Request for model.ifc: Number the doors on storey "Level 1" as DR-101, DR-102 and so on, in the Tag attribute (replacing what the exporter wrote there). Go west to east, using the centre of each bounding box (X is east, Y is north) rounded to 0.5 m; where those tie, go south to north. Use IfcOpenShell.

First a look at what the model holds.

```python
import ifcopenshell
import ifcopenshell.util.element
import ifcopenshell.util.placement

model = ifcopenshell.open("model.ifc")
print(model.schema)
storey = next(s for s in model.by_type("IfcBuildingStorey") if s.Name == "Level 1")
doors = [e for e in ifcopenshell.util.element.get_decomposition(storey) if e.is_a("IfcDoor")]
for e in sorted(doors, key=lambda e: e.id()):
    origin = ifcopenshell.util.placement.get_local_placement(e.ObjectPlacement)[:3, 3]
    print(e.id(), e.Tag, e.Name, origin.round(2) + 0.0, sep=" | ")
```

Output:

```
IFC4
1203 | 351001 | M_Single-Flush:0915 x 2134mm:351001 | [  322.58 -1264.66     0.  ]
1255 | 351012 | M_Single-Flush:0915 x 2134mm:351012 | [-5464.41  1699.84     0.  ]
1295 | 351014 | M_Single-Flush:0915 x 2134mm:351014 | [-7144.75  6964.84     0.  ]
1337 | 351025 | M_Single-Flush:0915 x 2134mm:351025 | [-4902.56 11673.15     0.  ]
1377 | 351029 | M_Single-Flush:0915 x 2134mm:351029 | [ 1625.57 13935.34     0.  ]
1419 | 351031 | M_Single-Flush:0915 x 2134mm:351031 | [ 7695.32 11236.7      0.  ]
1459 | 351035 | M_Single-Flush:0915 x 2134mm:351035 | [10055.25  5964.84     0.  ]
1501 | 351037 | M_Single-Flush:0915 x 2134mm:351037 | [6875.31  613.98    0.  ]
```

```python
import ifcopenshell
import ifcopenshell.geom
import ifcopenshell.util.element
import ifcopenshell.util.shape

model = ifcopenshell.open("model.ifc")
settings = ifcopenshell.geom.settings()
settings.set("use-world-coords", True)


def centre(element):
    shape = ifcopenshell.geom.create_shape(settings, element)
    return ifcopenshell.util.shape.get_bbox_centroid(shape.geometry)


storey = next(s for s in model.by_type("IfcBuildingStorey") if s.Name == "Level 1")
doors = [e for e in ifcopenshell.util.element.get_decomposition(storey) if e.is_a("IfcDoor")]

# Insertion points can sit at a corner or the storey origin, so sort by the geometry (in metres).
centres = {e: centre(e) for e in doors}
doors.sort(key=lambda e: (round(centres[e][0] / 0.5), centres[e][1]))

for i, e in enumerate(doors, start=1):
    number = f"DR-1{i:02d}"
    e.Tag = number
    print(e.id(), number)

model.write("model_v2.ifc")
```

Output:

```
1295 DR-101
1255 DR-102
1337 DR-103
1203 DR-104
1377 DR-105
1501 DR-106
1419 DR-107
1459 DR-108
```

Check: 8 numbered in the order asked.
